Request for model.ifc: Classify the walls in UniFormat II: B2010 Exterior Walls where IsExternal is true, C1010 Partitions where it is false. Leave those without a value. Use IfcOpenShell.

First a look at what the model holds.

```python
import ifcopenshell
import ifcopenshell.util.element

model = ifcopenshell.open("model.ifc")
print(model.schema)
print("classifications:", [c.Name for c in model.by_type("IfcClassification")])
values = [ifcopenshell.util.element.get_pset(e, "Pset_WallCommon", "IsExternal") for e in model.by_type("IfcWall")]
for value in (True, False, None):
    print("IsExternal", value, values.count(value))
```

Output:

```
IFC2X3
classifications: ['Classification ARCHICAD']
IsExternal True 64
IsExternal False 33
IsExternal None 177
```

```python
import ifcopenshell
import ifcopenshell.api.classification
import ifcopenshell.util.element

model = ifcopenshell.open("model.ifc")

# IFC2X3 requires Source and Edition and has no link from the project to the system.
system = model.create_entity("IfcClassification", Source="ASTM", Edition="E1557", Name="UniFormat II")

walls = model.by_type("IfcWall")
external = {e: ifcopenshell.util.element.get_pset(e, "Pset_WallCommon", "IsExternal") for e in walls}
for flag, code, name in ((True, "B2010", "Exterior Walls"), (False, "C1010", "Partitions")):
    products = [e for e in walls if external[e] is flag]
    ifcopenshell.api.classification.add_reference(
        model, products=products, classification=system, identification=code, name=name
    )
    print(code, len(products))

model.write("model_v2.ifc")
```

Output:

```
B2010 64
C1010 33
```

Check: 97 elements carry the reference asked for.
